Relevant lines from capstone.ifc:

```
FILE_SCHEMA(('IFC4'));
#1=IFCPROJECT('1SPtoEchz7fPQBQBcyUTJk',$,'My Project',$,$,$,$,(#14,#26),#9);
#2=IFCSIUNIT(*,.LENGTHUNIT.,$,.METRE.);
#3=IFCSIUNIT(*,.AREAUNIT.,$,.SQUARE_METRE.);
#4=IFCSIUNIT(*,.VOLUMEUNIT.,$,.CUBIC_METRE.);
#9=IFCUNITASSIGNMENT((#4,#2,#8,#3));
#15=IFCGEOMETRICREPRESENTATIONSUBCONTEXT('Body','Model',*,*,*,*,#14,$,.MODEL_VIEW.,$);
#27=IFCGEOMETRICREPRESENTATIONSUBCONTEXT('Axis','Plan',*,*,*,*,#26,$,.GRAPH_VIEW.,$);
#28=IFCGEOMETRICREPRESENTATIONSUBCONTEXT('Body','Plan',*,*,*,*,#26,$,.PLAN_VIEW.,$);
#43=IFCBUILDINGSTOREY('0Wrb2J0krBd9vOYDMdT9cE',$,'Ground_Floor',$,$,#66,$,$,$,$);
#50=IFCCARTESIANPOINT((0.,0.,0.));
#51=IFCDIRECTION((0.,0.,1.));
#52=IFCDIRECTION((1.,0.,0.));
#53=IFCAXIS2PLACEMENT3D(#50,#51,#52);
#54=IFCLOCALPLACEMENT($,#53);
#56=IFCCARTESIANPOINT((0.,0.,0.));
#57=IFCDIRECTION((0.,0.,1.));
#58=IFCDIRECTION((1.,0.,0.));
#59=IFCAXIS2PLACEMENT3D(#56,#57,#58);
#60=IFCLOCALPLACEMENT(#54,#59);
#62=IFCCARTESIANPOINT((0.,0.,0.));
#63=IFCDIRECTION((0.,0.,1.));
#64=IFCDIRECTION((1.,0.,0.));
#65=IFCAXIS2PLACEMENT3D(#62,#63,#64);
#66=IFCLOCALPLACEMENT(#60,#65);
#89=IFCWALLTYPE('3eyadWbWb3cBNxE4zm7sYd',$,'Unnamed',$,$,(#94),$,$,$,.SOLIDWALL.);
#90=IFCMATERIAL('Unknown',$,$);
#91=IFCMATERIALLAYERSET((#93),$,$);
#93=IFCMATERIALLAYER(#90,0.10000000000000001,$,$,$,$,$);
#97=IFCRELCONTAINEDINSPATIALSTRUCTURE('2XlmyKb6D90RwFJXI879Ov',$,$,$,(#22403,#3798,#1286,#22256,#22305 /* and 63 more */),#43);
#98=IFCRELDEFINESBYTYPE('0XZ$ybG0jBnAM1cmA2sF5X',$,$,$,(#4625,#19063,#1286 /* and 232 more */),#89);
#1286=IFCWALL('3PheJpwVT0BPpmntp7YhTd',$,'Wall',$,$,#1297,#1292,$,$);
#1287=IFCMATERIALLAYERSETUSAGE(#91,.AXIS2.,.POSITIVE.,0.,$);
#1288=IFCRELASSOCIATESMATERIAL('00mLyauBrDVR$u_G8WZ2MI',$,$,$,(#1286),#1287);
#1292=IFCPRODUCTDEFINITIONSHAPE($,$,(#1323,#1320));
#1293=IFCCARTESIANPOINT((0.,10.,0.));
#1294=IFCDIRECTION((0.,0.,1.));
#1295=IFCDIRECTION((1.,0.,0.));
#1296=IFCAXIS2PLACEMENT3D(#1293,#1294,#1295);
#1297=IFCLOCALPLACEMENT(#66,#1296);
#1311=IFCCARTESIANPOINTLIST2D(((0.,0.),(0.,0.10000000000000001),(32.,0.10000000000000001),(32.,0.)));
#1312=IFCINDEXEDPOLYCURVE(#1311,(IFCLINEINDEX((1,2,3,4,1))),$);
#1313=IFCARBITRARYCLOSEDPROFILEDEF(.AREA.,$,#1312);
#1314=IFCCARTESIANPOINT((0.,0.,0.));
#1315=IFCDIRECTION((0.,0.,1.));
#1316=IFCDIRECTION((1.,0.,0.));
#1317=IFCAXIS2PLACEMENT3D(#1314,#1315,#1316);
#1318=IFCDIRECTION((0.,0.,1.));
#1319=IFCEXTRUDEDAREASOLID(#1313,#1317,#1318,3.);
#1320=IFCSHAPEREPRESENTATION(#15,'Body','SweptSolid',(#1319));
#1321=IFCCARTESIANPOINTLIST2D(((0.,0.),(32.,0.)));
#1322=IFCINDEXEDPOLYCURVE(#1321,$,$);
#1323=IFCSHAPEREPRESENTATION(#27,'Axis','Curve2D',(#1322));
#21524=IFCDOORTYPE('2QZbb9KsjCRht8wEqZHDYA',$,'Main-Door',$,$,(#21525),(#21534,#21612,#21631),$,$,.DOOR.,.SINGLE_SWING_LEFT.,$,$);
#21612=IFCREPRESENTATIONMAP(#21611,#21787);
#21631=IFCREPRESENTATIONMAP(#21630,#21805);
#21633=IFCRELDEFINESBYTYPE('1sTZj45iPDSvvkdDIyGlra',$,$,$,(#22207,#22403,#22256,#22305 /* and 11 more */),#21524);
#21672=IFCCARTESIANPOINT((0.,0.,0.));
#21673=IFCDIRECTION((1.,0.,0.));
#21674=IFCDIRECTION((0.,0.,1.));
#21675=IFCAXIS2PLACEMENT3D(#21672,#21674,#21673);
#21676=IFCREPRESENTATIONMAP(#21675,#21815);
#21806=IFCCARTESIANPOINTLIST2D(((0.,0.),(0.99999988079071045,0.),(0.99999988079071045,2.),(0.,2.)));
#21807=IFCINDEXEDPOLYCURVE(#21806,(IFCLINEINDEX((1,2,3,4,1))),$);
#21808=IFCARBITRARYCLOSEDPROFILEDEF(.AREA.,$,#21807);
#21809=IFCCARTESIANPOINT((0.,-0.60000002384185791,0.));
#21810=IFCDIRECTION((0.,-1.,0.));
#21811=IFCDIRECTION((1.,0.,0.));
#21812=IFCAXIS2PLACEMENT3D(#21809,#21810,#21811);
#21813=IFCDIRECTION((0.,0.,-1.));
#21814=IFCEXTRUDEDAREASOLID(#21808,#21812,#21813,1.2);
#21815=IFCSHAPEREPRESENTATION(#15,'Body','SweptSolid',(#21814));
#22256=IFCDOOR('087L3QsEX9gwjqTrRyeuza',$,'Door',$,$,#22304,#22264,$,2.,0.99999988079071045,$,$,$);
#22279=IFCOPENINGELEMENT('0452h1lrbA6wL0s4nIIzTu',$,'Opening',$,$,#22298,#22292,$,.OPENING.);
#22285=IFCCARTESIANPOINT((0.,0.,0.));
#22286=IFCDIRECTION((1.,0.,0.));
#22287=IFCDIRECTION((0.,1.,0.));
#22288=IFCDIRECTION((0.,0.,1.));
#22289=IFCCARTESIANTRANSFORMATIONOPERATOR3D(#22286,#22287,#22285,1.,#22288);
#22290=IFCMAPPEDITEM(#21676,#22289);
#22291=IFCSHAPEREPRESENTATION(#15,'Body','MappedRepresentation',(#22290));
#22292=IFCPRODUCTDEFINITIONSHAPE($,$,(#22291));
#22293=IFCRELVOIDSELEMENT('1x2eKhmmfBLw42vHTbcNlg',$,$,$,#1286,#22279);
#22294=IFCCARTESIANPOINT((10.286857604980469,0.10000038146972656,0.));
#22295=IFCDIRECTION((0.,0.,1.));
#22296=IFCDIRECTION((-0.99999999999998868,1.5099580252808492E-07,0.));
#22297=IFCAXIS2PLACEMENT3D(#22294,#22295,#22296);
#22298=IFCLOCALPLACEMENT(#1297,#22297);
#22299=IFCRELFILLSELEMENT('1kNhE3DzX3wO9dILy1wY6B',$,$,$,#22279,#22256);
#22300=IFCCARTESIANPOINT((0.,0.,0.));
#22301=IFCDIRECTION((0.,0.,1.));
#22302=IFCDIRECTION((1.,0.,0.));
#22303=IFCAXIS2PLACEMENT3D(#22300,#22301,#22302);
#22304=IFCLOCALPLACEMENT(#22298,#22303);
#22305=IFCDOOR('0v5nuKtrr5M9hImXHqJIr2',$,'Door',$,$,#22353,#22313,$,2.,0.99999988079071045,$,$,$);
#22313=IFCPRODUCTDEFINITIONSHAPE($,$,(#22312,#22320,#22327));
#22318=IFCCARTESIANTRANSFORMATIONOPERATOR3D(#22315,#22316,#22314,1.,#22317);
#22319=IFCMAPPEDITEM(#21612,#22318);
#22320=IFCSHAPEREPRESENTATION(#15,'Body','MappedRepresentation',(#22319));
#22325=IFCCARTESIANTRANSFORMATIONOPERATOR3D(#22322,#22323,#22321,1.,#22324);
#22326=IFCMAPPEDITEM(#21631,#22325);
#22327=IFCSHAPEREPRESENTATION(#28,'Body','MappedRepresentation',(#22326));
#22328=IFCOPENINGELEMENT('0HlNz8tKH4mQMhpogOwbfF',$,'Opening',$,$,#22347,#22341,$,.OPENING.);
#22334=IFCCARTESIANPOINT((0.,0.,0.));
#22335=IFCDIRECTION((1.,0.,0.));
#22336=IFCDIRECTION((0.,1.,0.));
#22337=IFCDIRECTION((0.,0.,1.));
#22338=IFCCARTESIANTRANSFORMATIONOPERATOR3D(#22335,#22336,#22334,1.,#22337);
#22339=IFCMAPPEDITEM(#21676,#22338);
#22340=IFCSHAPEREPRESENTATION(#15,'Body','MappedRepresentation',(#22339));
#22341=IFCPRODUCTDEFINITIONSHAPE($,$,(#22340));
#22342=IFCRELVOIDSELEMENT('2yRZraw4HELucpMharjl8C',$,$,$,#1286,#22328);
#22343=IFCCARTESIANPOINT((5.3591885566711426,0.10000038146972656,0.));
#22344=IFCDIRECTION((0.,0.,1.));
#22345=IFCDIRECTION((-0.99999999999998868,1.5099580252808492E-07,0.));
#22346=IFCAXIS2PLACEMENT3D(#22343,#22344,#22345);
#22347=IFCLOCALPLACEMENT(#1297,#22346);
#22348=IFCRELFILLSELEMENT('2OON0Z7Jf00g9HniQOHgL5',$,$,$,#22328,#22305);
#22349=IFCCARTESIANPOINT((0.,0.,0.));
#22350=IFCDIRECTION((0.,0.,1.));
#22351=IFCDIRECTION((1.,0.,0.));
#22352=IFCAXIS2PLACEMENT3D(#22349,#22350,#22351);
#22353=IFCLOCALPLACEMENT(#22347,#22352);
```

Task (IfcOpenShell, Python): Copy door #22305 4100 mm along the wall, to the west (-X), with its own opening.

```python
import ifcopenshell
import ifcopenshell.api.feature
import ifcopenshell.api.geometry
import ifcopenshell.api.root
import ifcopenshell.geom
import ifcopenshell.util.element
import ifcopenshell.util.placement
import ifcopenshell.util.shape

model = ifcopenshell.open("capstone.ifc")
settings = ifcopenshell.geom.settings()


def volume(element):
    """Net volume in cubic metres, openings subtracted."""
    shape = ifcopenshell.geom.create_shape(settings, element)
    return ifcopenshell.util.shape.get_volume(shape.geometry)


door = model.by_guid("0v5nuKtrr5M9hImXHqJIr2")
opening = door.FillsVoids[0].RelatingOpeningElement
wall = opening.VoidsElements[0].RelatingBuildingElement
before = volume(wall)
shift = ifcopenshell.util.placement.get_local_placement(wall.ObjectPlacement)[:3, 0] * -4.1

# copy_class copies the void relationship, type, container and properties, but no geometry.
new_opening = ifcopenshell.api.root.copy_class(model, product=opening)
new_opening.Representation = ifcopenshell.util.element.copy_deep(
    model, opening.Representation, exclude=["IfcGeometricRepresentationContext", "IfcRepresentationMap"]
)
new_door = ifcopenshell.api.root.copy_class(model, product=door)
new_door.Representation = ifcopenshell.util.element.copy_deep(
    model, door.Representation, exclude=["IfcGeometricRepresentationContext", "IfcRepresentationMap"]
)
ifcopenshell.api.feature.add_filling(model, opening=new_opening, element=new_door)

for old, new in ((opening, new_opening), (door, new_door)):
    matrix = ifcopenshell.util.placement.get_local_placement(old.ObjectPlacement)
    matrix[:3, 3] += shift
    ifcopenshell.api.geometry.edit_object_placement(model, product=new, matrix=matrix, is_si=False)

after = volume(wall)

print(f"wall volume {before:.3f} -> {after:.3f} m3")

model.write("capstone_edited.ifc")
```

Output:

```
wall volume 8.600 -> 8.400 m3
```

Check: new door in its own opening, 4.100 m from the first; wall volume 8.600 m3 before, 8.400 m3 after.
